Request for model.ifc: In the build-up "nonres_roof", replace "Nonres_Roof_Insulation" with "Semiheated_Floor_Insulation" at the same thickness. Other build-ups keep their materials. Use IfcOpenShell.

First a look at what the model holds.

```python
import ifcopenshell
import ifcopenshell.util.element

model = ifcopenshell.open("model.ifc")
print(model.schema)
for layer_set in model.by_type("IfcMaterialLayerSet"):
    if layer_set.LayerSetName == "nonres_roof":
        for layer in layer_set.MaterialLayers:
            print(layer.id(), layer.Material and layer.Material.Name, layer.LayerThickness, sep=" | ")
        print(len(ifcopenshell.util.element.get_elements_by_material(model, layer_set)), "elements and types use it")
print(sorted(m.Name for m in model.by_type("IfcMaterial") if m.Name)[:60])
```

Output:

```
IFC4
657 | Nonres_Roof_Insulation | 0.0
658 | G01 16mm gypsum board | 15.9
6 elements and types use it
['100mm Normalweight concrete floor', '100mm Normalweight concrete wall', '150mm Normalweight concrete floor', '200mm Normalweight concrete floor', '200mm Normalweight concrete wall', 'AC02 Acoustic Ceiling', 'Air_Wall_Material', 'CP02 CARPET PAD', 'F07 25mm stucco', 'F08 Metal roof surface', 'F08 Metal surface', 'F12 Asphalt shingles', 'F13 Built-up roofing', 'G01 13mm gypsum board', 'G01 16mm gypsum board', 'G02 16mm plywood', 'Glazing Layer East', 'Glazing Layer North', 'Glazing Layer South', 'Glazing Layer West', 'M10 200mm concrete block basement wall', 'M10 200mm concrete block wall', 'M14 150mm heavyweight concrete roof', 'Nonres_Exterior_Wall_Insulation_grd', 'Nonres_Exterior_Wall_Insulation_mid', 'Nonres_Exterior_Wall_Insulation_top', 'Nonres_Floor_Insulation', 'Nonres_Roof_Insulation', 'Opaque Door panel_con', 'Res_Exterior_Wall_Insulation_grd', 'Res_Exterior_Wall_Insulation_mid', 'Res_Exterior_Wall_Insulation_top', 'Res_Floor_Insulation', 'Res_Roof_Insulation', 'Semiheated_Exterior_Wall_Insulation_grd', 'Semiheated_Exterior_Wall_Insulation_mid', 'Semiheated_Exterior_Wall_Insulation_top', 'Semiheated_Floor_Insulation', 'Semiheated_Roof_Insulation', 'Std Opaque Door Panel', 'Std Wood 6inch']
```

```python
import ifcopenshell
import ifcopenshell.api.material

model = ifcopenshell.open("model.ifc")

layer_set = next(s for s in model.by_type("IfcMaterialLayerSet") if s.LayerSetName == "nonres_roof")
layer = next(l for l in layer_set.MaterialLayers if l.Material and l.Material.Name == "Nonres_Roof_Insulation")
material = next(m for m in model.by_type("IfcMaterial") if m.Name == "Semiheated_Floor_Insulation")

# Point this one layer at the other material; renaming the old one would change it everywhere.
ifcopenshell.api.material.edit_layer(model, layer=layer, attributes={}, material=material)

print([l.Material.Name if l.Material else None for l in layer_set.MaterialLayers])

model.write("model-out.ifc")
```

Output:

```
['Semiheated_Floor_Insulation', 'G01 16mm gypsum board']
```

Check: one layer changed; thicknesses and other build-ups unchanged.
